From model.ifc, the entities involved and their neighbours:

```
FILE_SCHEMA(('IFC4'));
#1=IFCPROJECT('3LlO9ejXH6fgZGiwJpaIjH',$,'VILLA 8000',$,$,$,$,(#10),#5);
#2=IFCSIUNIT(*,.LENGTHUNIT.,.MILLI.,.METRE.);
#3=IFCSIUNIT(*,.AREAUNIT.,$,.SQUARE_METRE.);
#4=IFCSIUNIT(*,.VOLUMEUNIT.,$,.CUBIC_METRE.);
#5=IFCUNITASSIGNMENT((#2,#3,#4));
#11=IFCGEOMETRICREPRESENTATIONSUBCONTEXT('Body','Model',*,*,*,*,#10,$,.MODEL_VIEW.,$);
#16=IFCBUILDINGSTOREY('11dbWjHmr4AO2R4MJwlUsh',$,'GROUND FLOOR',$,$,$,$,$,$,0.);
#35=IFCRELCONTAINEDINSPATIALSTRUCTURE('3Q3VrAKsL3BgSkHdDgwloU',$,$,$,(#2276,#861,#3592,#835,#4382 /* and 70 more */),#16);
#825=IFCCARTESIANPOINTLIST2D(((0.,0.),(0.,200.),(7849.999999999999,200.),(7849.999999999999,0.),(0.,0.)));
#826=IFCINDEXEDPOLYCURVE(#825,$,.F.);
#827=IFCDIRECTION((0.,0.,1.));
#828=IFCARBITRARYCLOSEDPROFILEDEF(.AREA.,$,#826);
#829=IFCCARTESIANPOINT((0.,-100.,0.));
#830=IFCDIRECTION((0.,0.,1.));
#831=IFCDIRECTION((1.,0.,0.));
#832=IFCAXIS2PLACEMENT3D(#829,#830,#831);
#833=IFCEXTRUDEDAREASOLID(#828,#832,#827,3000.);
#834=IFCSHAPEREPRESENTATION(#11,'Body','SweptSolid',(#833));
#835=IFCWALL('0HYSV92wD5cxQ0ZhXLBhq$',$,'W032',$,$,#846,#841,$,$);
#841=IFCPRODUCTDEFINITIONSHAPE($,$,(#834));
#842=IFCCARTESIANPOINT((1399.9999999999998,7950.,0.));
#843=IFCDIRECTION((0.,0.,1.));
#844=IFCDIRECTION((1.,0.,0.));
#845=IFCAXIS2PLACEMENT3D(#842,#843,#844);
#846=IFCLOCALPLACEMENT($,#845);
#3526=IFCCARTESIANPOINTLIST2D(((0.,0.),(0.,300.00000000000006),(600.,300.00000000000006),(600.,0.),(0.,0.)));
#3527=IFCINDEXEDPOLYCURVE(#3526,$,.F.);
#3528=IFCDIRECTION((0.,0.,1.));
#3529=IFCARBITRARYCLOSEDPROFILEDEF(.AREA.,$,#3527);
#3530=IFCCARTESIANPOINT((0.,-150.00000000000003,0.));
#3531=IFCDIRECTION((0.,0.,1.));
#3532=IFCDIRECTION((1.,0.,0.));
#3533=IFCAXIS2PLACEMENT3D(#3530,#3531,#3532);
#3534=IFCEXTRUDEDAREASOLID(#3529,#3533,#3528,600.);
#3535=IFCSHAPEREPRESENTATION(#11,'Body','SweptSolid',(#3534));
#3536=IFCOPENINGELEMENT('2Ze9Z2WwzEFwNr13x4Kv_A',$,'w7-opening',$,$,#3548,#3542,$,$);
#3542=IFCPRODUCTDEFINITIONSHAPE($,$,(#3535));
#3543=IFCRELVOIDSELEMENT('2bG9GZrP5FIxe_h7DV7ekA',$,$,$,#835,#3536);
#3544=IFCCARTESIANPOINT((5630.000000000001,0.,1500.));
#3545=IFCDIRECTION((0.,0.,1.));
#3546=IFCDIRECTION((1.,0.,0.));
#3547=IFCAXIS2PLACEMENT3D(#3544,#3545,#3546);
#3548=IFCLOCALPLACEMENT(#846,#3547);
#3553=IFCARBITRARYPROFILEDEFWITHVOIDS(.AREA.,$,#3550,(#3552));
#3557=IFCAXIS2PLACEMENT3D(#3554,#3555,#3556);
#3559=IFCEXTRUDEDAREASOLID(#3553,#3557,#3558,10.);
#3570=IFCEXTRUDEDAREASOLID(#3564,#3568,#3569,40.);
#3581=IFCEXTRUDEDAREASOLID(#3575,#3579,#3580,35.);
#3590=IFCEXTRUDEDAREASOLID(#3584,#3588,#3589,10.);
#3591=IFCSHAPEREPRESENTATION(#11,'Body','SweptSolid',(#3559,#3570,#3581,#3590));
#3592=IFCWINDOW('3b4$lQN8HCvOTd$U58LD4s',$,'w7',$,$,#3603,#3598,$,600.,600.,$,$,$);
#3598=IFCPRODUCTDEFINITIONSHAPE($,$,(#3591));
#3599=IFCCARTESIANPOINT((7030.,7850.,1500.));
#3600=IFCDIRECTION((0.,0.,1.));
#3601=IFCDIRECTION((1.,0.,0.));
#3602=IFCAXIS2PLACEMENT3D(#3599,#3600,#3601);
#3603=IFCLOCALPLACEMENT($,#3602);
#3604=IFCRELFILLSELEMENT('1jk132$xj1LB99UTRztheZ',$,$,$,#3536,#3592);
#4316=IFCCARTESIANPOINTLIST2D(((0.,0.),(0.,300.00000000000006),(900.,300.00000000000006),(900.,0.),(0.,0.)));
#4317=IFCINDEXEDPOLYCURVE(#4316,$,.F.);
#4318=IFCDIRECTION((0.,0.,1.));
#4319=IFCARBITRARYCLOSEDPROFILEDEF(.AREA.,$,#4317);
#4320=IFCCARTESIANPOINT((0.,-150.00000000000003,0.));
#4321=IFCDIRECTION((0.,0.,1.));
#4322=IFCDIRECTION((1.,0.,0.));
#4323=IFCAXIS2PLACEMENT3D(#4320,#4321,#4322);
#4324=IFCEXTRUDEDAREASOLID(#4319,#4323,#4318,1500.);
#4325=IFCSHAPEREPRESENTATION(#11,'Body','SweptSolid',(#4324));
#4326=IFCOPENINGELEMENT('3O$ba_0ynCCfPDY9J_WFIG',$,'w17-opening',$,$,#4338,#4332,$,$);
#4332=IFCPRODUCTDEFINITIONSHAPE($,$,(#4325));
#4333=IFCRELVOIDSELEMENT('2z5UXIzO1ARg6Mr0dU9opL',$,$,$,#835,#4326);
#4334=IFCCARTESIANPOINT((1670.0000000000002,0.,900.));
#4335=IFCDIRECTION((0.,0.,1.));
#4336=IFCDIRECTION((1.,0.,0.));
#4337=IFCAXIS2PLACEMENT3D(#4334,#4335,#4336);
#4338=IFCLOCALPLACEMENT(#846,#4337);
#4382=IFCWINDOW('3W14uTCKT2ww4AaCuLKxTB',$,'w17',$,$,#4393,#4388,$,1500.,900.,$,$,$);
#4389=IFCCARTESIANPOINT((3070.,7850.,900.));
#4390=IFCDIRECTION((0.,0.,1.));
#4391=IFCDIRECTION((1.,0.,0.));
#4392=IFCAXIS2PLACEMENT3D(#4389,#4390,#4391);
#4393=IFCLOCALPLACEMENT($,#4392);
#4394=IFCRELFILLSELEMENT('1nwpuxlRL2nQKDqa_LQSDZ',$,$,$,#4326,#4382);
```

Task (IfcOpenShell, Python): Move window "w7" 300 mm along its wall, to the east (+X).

```python
import ifcopenshell
import ifcopenshell.api.geometry
import ifcopenshell.util.placement

model = ifcopenshell.open("model.ifc")

window = model.by_guid("3b4$lQN8HCvOTd$U58LD4s")
opening = window.FillsVoids[0].RelatingOpeningElement
wall = opening.VoidsElements[0].RelatingBuildingElement

wall_matrix = ifcopenshell.util.placement.get_local_placement(wall.ObjectPlacement)
shift = wall_matrix[:3, 0] * 300.0
before = ifcopenshell.util.placement.get_local_placement(window.ObjectPlacement)[:3, 3].copy()

# The window is not placed relative to its opening, so move both.
for product in (opening, window):
    matrix = ifcopenshell.util.placement.get_local_placement(product.ObjectPlacement)
    matrix[:3, 3] += shift
    ifcopenshell.api.geometry.edit_object_placement(model, product=product, matrix=matrix, is_si=False)

after = ifcopenshell.util.placement.get_local_placement(window.ObjectPlacement)[:3, 3]
print("window moved by", (after - before).round(3) + 0.0)

model.write("model_v2.ifc")
```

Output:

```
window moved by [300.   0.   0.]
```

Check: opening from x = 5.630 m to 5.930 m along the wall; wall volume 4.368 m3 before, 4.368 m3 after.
